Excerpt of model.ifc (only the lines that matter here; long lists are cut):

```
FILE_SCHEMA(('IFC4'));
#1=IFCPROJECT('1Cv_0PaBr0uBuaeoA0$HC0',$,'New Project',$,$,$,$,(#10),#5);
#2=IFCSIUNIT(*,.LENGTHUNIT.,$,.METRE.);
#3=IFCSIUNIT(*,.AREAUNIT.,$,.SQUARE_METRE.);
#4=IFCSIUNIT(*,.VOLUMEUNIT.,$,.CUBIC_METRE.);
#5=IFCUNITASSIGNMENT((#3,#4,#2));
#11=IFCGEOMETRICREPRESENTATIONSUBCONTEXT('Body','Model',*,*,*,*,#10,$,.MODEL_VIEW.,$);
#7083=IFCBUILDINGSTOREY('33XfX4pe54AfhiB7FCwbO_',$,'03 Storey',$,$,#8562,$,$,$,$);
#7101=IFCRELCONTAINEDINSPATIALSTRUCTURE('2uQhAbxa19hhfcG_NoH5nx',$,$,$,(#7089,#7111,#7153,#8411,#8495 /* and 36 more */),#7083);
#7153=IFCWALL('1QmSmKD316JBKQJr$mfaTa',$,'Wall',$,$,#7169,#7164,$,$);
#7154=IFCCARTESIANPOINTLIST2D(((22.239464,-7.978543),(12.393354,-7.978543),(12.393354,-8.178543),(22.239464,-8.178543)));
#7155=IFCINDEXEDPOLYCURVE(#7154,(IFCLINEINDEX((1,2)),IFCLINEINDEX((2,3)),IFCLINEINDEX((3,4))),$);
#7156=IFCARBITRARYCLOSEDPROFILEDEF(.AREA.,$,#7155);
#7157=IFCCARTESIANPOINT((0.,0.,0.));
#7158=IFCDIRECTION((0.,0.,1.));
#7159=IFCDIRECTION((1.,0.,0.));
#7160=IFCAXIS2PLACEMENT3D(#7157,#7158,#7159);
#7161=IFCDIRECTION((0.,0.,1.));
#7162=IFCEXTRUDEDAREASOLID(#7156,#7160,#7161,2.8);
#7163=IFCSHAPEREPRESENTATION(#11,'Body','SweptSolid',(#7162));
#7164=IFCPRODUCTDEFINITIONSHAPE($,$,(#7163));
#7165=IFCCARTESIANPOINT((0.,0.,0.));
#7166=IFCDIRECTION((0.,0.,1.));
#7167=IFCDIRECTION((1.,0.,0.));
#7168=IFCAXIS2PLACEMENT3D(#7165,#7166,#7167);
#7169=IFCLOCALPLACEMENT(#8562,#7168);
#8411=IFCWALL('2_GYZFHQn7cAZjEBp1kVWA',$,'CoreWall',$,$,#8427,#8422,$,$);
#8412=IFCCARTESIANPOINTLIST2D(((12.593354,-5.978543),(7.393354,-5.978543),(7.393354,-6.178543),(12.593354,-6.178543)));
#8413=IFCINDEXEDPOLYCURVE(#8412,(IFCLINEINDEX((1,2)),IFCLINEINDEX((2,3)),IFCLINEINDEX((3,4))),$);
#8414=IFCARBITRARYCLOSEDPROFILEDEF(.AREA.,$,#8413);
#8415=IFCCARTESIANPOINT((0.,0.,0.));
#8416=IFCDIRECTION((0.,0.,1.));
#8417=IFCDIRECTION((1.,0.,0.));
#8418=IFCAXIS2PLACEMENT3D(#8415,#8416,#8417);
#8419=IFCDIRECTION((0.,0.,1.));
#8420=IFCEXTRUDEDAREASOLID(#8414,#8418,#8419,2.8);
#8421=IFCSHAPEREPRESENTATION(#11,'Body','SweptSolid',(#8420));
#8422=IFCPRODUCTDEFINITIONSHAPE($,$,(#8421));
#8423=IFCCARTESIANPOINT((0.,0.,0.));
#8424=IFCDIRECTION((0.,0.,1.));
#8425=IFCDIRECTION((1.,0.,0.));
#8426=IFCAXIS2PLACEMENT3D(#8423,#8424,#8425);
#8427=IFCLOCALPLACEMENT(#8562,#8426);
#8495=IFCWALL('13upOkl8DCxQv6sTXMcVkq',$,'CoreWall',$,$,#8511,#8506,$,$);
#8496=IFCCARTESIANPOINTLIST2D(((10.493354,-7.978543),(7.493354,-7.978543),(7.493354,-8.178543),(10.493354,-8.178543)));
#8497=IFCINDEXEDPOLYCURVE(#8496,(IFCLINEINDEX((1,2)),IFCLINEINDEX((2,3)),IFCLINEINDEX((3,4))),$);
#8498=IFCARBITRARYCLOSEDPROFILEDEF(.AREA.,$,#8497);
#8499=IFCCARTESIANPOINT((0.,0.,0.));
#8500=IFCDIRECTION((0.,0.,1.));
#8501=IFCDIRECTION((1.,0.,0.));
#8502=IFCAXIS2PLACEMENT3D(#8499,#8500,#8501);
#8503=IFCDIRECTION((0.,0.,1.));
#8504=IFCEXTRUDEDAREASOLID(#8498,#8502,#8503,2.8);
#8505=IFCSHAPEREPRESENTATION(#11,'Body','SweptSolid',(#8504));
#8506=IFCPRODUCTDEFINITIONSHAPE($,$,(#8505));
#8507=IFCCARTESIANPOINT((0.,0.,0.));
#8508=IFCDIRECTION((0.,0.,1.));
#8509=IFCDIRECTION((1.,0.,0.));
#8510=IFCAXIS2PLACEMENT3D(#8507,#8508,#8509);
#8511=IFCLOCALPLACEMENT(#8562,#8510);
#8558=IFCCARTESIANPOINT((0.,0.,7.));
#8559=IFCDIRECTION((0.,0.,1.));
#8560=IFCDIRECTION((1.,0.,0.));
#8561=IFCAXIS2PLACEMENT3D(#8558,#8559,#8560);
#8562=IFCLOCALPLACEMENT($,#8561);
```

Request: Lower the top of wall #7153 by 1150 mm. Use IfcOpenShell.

```python
import ifcopenshell
import ifcopenshell.geom
import ifcopenshell.util.representation
import ifcopenshell.util.shape
import ifcopenshell.util.unit

model = ifcopenshell.open("model.ifc")
unit_scale = ifcopenshell.util.unit.calculate_unit_scale(model)
settings = ifcopenshell.geom.settings()


def volume(element):
    """Net volume in cubic metres, openings subtracted."""
    shape = ifcopenshell.geom.create_shape(settings, element)
    return ifcopenshell.util.shape.get_volume(shape.geometry)


wall = model.by_id(7153)
before = volume(wall)

body = ifcopenshell.util.representation.get_representation(wall, "Model", "Body")
solid = body.Items[0]
old_height = solid.Depth
solid.Depth -= 1.15 / unit_scale
after = volume(wall)

print(f"height {old_height:g} -> {solid.Depth:g}, volume {before:.3f} -> {after:.3f} m3")

model.write("model_updated.ifc")
```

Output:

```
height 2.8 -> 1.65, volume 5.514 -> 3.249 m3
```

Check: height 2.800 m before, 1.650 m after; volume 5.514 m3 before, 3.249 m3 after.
